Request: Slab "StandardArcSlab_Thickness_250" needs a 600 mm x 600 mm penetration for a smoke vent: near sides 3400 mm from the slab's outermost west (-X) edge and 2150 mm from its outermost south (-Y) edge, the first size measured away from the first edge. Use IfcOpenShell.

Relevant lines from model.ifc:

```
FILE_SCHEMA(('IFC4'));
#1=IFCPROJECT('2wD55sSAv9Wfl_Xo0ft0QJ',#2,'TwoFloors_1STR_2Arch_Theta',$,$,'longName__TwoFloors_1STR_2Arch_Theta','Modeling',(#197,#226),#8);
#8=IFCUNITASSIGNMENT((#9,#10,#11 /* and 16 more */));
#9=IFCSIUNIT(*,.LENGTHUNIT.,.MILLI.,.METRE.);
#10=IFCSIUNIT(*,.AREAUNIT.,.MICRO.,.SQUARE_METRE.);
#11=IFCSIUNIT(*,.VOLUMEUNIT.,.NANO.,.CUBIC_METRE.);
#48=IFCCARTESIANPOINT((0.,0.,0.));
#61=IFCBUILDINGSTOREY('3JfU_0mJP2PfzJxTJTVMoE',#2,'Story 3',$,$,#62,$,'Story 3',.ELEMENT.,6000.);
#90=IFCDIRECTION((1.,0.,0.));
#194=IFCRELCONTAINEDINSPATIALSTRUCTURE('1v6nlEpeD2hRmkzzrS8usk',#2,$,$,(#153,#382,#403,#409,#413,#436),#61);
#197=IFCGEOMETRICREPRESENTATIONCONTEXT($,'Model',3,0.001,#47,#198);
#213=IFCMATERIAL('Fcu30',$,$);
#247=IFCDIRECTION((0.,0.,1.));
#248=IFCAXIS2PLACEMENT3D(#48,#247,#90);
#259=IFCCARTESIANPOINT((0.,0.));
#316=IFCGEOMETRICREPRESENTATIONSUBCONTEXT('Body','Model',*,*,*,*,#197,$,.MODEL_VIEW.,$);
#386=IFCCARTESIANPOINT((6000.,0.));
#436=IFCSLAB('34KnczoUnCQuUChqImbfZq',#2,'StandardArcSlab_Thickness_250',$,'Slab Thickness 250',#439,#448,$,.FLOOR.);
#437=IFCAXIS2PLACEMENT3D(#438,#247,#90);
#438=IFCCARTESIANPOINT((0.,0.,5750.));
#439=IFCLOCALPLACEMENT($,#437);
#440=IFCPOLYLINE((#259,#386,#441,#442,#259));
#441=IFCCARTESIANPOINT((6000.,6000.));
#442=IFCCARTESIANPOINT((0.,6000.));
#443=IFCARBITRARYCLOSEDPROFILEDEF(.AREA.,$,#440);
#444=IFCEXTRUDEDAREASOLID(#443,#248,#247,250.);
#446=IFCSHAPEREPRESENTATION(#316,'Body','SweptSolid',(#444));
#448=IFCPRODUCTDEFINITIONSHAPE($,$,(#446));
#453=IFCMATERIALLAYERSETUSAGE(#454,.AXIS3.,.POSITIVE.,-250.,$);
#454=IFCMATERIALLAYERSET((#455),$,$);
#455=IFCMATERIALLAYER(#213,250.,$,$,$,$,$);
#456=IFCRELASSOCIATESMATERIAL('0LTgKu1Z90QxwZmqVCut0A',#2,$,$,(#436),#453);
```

```python
import numpy as np
import ifcopenshell
import ifcopenshell.api.feature
import ifcopenshell.api.geometry
import ifcopenshell.api.root
import ifcopenshell.geom
import ifcopenshell.util.placement
import ifcopenshell.util.representation
import ifcopenshell.util.shape
import ifcopenshell.util.unit

model = ifcopenshell.open("model.ifc")
unit_scale = ifcopenshell.util.unit.calculate_unit_scale(model)
settings = ifcopenshell.geom.settings()


def volume(element):
    """Net volume in cubic metres, openings subtracted."""
    shape = ifcopenshell.geom.create_shape(settings, element)
    return ifcopenshell.util.shape.get_volume(shape.geometry)


slab = model.by_guid("34KnczoUnCQuUChqImbfZq")
before = volume(slab)

# Extent in the slab's own axes, in metres. The edges named are its -X and -Y sides.
slab_shape = ifcopenshell.geom.create_shape(settings, slab)
vertices = ifcopenshell.util.shape.get_vertices(slab_shape.geometry)
x_min, y_min, bottom = vertices.min(axis=0)
top = vertices[:, 2].max()

opening = ifcopenshell.api.root.create_entity(model, ifc_class="IfcOpeningElement", name="Smoke vent opening", predefined_type="OPENING")
context = ifcopenshell.util.representation.get_context(model, "Model", "Body", "MODEL_VIEW")
width, depth = 0.6, 0.6
outline = [(0.0, 0.0), (width, 0.0), (width, depth), (0.0, depth), (0.0, 0.0)]
# Overshoot both faces by 50 mm so the cut is clean.
shape = ifcopenshell.api.geometry.add_slab_representation(
    model, context=context, depth=top - bottom + 0.1, polyline=outline
)
ifcopenshell.api.geometry.assign_representation(model, product=opening, representation=shape)

matrix = ifcopenshell.util.placement.get_local_placement(slab.ObjectPlacement)
matrix[:, 3] = matrix @ np.append(np.array([x_min + 3.4, y_min + 2.15, bottom - 0.05]) / unit_scale, 1.0)
ifcopenshell.api.geometry.edit_object_placement(model, product=opening, matrix=matrix, is_si=False)
ifcopenshell.api.feature.add_feature(model, feature=opening, element=slab)

after = volume(slab)

print(f"slab volume {before:.3f} -> {after:.3f} m3")

model.write("model-out.ifc")
```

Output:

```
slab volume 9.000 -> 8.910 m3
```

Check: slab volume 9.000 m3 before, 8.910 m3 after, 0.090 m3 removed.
